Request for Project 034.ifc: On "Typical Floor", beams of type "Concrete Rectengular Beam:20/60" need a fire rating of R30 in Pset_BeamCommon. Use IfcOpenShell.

First a look at what the model holds.

```python
import ifcopenshell
import ifcopenshell.util.element

model = ifcopenshell.open("Project 034.ifc")
print(model.schema)
storey = next(s for s in model.by_type("IfcBuildingStorey") if s.Name == "Typical Floor")
beams = [e for e in ifcopenshell.util.element.get_decomposition(storey) if e.is_a("IfcBeam")]
seen = {}
for e in beams:
    element_type = ifcopenshell.util.element.get_type(e)
    key = (element_type.Name if element_type != e and element_type else None, ifcopenshell.util.element.get_pset(e, "Pset_BeamCommon", "FireRating"))
    seen[key] = seen.get(key, 0) + 1
for (name, value), count in sorted(seen.items(), key=str):
    print(count, "x", name, "|", value)
```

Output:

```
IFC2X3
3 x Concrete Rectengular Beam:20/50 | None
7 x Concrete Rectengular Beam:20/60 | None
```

```python
import ifcopenshell
import ifcopenshell.api.pset
import ifcopenshell.util.element

model = ifcopenshell.open("Project 034.ifc")

storey = next(s for s in model.by_type("IfcBuildingStorey") if s.Name == "Typical Floor")
beams = [e for e in ifcopenshell.util.element.get_decomposition(storey) if e.is_a("IfcBeam")]

count = 0
for e in beams:
    element_type = ifcopenshell.util.element.get_type(e)
    if element_type in (None, e) or element_type.Name != "Concrete Rectengular Beam:20/60":
        continue
    # add_pset returns the element's existing set when there is one.
    pset = ifcopenshell.api.pset.add_pset(model, product=e, name="Pset_BeamCommon")
    ifcopenshell.api.pset.edit_pset(model, pset=pset, properties={"FireRating": "R30"})
    count += 1

print(count, "beams updated")

model.write("Project 034-out.ifc")
```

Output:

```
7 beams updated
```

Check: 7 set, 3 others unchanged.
